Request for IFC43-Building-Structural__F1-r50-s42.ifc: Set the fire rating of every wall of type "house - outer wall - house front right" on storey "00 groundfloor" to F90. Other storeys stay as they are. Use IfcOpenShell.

First a look at what the model holds.

```python
import ifcopenshell
import ifcopenshell.util.element

model = ifcopenshell.open("IFC43-Building-Structural__F1-r50-s42.ifc")
print(model.schema)
storey = next(s for s in model.by_type("IfcBuildingStorey") if s.Name == "00 groundfloor")
walls = [e for e in ifcopenshell.util.element.get_decomposition(storey) if e.is_a("IfcWall")]
seen = {}
for e in walls:
    element_type = ifcopenshell.util.element.get_type(e)
    key = (element_type.Name if element_type != e and element_type else None, ifcopenshell.util.element.get_pset(e, "Pset_WallCommon", "FireRating"))
    seen[key] = seen.get(key, 0) + 1
for (name, value), count in sorted(seen.items(), key=str):
    print(count, "x", name, "|", value)
```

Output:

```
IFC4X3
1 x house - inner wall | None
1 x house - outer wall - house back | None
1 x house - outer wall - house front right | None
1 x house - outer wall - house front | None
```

```python
import ifcopenshell
import ifcopenshell.api.pset
import ifcopenshell.util.element

model = ifcopenshell.open("IFC43-Building-Structural__F1-r50-s42.ifc")

storey = next(s for s in model.by_type("IfcBuildingStorey") if s.Name == "00 groundfloor")
walls = [e for e in ifcopenshell.util.element.get_decomposition(storey) if e.is_a("IfcWall")]

count = 0
for e in walls:
    element_type = ifcopenshell.util.element.get_type(e)
    if element_type in (None, e) or element_type.Name != "house - outer wall - house front right":
        continue
    # add_pset returns the element's existing set when there is one.
    pset = ifcopenshell.api.pset.add_pset(model, product=e, name="Pset_WallCommon")
    ifcopenshell.api.pset.edit_pset(model, pset=pset, properties={"FireRating": "F90"})
    count += 1

print(count, "walls updated")

model.write("IFC43-Building-Structural__F1-r50-s42_v2.ifc")
```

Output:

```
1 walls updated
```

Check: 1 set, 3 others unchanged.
